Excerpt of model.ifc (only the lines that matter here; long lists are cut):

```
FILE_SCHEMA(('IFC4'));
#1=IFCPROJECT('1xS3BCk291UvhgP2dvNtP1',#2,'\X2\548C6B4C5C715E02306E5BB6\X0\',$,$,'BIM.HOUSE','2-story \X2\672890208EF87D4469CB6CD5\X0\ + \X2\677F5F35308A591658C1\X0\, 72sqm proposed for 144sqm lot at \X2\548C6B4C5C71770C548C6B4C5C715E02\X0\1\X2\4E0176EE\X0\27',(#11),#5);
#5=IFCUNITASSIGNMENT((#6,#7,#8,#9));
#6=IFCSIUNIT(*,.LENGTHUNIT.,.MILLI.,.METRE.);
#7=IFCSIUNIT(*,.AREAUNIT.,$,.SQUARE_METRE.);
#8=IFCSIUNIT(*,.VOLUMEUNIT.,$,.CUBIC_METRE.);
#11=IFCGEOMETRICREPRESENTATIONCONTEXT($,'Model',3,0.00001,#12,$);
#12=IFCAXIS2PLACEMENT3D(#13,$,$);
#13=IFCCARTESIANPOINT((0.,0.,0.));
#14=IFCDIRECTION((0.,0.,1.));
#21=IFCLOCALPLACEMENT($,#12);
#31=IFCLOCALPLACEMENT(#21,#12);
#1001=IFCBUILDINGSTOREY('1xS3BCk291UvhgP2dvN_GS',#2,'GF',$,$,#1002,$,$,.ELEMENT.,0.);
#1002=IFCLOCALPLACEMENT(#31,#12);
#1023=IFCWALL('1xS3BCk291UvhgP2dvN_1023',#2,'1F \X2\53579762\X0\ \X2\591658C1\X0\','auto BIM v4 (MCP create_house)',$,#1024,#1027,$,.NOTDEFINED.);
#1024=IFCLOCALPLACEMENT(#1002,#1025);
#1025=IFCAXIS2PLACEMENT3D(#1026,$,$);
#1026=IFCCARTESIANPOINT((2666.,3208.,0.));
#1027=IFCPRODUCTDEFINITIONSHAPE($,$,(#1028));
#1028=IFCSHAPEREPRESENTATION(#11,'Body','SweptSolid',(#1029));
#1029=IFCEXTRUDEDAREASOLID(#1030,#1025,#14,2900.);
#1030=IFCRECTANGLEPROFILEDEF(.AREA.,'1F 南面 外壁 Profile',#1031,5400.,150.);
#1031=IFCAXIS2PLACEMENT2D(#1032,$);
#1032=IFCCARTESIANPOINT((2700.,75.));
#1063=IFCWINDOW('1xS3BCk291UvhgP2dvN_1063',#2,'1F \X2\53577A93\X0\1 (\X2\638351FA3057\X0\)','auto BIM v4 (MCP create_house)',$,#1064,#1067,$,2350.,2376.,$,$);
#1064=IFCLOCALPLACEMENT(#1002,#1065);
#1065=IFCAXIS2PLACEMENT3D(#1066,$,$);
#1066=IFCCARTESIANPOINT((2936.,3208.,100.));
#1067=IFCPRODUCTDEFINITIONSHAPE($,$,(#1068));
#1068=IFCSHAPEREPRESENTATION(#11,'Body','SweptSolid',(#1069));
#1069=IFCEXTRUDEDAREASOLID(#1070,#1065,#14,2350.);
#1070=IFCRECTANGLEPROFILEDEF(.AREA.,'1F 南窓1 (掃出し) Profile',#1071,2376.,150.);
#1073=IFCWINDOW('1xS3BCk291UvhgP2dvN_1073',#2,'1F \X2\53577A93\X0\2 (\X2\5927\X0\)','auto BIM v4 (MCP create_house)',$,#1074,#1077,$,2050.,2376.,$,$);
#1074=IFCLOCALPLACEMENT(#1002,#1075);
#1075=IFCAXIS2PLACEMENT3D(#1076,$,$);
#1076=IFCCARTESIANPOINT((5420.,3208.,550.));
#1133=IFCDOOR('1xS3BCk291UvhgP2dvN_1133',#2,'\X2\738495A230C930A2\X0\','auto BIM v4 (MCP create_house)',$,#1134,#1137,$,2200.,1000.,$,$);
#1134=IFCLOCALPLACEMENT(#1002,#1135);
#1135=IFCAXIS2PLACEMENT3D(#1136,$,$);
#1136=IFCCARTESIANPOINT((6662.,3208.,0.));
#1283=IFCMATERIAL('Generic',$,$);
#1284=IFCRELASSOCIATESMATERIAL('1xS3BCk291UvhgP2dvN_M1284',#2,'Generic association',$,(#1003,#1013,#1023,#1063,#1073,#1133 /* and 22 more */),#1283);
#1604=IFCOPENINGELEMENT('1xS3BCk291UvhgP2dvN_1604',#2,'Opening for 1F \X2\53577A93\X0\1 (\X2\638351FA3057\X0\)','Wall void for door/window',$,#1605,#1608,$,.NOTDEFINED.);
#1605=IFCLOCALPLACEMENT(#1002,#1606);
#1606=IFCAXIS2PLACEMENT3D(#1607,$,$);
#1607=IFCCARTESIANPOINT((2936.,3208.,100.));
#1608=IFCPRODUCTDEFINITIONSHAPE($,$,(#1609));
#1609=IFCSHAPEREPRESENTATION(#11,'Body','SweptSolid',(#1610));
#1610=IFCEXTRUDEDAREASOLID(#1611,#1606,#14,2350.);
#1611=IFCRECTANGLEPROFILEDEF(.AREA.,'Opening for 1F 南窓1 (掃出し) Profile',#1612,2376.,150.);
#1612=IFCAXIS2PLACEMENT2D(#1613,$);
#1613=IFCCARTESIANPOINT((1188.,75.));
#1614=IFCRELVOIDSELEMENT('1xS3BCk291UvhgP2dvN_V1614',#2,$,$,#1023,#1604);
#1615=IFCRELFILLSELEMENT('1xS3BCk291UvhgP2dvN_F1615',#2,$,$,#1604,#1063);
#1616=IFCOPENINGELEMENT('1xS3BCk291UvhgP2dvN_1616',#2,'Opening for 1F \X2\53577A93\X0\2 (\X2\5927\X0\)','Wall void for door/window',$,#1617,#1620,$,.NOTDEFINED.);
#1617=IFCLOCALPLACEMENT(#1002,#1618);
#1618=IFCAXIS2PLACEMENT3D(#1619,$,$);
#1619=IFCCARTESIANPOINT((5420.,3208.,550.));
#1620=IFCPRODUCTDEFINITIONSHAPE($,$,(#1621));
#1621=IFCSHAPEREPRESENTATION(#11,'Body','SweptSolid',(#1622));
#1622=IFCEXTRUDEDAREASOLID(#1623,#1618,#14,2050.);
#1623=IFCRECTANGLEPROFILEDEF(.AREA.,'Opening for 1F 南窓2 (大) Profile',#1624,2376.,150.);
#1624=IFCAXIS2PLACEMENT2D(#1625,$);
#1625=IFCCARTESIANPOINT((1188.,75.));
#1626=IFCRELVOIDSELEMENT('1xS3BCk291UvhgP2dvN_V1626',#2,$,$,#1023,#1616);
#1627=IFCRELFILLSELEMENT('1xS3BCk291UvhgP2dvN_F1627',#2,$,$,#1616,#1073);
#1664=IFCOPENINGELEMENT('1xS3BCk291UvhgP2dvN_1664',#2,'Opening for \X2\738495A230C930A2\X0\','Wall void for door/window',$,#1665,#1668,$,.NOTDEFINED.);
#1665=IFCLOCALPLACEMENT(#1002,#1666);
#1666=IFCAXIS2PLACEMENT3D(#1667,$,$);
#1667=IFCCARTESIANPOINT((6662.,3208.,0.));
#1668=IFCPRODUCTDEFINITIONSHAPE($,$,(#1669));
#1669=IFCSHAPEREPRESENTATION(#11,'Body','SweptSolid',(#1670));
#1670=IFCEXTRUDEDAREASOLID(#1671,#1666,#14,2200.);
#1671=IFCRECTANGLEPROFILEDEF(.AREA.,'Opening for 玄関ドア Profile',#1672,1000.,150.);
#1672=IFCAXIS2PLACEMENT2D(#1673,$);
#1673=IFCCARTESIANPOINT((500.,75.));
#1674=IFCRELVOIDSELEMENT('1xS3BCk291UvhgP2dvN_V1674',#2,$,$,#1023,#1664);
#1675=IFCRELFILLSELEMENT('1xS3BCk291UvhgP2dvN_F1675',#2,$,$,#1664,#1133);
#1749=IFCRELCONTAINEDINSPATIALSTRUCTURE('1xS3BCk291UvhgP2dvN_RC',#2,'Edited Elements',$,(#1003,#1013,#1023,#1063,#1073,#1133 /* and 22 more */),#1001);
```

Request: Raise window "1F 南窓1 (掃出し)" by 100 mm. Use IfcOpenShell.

```python
import numpy as np
import ifcopenshell
import ifcopenshell.api.geometry
import ifcopenshell.util.placement
import ifcopenshell.util.unit

model = ifcopenshell.open("model.ifc")
unit_scale = ifcopenshell.util.unit.calculate_unit_scale(model)

window = model.by_guid("1xS3BCk291UvhgP2dvN_1063")
opening = window.FillsVoids[0].RelatingOpeningElement
dz = 0.1 / unit_scale

shift = np.array([0.0, 0.0, dz])
# The window is not placed relative to its opening, so move both.
for product in (opening, window):
    matrix = ifcopenshell.util.placement.get_local_placement(product.ObjectPlacement)
    matrix[:3, 3] += shift
    ifcopenshell.api.geometry.edit_object_placement(model, product=product, matrix=matrix, is_si=False)

print(f"moved by {dz * unit_scale:+.3f} m")

model.write("model_rev.ifc")
```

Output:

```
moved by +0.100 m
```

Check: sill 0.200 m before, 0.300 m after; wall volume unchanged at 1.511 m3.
